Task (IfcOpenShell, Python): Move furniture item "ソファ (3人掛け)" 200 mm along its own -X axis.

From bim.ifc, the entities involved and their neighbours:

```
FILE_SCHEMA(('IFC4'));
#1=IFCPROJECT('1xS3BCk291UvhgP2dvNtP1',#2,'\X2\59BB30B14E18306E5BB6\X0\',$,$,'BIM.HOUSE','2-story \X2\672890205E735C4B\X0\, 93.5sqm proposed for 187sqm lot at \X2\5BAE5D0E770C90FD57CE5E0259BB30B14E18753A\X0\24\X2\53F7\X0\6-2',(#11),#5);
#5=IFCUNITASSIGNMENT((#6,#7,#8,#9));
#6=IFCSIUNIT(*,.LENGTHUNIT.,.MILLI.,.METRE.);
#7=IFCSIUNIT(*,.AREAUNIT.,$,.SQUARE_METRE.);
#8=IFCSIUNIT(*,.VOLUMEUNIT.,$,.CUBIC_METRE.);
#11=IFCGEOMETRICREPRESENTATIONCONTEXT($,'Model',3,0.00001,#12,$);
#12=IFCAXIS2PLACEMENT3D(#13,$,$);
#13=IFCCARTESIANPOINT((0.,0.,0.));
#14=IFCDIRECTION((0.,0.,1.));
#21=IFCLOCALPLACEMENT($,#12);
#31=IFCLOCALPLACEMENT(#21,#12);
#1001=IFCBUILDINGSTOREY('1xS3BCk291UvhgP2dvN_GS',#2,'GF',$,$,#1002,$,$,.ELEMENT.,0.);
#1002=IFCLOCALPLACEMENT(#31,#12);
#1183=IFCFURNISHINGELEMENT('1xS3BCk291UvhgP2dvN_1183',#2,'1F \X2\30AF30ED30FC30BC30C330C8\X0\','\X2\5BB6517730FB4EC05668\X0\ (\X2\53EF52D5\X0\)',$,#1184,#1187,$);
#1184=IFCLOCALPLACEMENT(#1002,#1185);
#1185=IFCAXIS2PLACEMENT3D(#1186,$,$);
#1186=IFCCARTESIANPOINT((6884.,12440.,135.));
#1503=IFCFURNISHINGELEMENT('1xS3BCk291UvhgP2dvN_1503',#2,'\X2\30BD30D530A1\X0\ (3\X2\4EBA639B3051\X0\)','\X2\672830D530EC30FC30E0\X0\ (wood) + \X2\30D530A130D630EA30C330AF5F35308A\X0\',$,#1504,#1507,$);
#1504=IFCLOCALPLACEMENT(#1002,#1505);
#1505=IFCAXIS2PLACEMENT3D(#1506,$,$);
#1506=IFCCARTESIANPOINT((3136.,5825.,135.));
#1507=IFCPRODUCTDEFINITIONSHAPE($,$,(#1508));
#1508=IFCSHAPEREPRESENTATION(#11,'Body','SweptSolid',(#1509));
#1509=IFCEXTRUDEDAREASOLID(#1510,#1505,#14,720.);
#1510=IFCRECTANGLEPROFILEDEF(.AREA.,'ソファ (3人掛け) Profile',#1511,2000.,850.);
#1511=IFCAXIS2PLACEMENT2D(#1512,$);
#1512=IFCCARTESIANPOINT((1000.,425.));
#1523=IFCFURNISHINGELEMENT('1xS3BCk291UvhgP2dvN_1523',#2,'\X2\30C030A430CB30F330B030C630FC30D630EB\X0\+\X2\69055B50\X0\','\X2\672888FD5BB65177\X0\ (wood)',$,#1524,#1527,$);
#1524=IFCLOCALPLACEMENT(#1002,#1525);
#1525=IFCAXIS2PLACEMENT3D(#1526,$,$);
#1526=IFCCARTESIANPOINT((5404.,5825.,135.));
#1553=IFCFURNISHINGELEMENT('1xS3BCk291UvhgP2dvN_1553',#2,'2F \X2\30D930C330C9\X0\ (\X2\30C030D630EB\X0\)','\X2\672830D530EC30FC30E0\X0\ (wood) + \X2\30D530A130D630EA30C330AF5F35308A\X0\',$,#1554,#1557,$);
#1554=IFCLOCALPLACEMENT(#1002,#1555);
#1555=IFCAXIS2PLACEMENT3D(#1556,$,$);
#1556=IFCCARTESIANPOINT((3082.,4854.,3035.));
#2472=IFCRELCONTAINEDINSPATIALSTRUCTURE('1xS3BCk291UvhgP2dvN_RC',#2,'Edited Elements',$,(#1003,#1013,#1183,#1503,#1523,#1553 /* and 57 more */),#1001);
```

```python
import ifcopenshell
import ifcopenshell.api.geometry
import ifcopenshell.util.placement

model = ifcopenshell.open("bim.ifc")

item = model.by_guid("1xS3BCk291UvhgP2dvN_1503")
matrix = ifcopenshell.util.placement.get_local_placement(item.ObjectPlacement)
matrix[:3, 3] -= matrix[:3, 0] * 200.0
ifcopenshell.api.geometry.edit_object_placement(model, product=item, matrix=matrix, is_si=False)

print(ifcopenshell.util.placement.get_local_placement(item.ObjectPlacement).round(3) + 0.0)

model.write("bim_updated.ifc")
```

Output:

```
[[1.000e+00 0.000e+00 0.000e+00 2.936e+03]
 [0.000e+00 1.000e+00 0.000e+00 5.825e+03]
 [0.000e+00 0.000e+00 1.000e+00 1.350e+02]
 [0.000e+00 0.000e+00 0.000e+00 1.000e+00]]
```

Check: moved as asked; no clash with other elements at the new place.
